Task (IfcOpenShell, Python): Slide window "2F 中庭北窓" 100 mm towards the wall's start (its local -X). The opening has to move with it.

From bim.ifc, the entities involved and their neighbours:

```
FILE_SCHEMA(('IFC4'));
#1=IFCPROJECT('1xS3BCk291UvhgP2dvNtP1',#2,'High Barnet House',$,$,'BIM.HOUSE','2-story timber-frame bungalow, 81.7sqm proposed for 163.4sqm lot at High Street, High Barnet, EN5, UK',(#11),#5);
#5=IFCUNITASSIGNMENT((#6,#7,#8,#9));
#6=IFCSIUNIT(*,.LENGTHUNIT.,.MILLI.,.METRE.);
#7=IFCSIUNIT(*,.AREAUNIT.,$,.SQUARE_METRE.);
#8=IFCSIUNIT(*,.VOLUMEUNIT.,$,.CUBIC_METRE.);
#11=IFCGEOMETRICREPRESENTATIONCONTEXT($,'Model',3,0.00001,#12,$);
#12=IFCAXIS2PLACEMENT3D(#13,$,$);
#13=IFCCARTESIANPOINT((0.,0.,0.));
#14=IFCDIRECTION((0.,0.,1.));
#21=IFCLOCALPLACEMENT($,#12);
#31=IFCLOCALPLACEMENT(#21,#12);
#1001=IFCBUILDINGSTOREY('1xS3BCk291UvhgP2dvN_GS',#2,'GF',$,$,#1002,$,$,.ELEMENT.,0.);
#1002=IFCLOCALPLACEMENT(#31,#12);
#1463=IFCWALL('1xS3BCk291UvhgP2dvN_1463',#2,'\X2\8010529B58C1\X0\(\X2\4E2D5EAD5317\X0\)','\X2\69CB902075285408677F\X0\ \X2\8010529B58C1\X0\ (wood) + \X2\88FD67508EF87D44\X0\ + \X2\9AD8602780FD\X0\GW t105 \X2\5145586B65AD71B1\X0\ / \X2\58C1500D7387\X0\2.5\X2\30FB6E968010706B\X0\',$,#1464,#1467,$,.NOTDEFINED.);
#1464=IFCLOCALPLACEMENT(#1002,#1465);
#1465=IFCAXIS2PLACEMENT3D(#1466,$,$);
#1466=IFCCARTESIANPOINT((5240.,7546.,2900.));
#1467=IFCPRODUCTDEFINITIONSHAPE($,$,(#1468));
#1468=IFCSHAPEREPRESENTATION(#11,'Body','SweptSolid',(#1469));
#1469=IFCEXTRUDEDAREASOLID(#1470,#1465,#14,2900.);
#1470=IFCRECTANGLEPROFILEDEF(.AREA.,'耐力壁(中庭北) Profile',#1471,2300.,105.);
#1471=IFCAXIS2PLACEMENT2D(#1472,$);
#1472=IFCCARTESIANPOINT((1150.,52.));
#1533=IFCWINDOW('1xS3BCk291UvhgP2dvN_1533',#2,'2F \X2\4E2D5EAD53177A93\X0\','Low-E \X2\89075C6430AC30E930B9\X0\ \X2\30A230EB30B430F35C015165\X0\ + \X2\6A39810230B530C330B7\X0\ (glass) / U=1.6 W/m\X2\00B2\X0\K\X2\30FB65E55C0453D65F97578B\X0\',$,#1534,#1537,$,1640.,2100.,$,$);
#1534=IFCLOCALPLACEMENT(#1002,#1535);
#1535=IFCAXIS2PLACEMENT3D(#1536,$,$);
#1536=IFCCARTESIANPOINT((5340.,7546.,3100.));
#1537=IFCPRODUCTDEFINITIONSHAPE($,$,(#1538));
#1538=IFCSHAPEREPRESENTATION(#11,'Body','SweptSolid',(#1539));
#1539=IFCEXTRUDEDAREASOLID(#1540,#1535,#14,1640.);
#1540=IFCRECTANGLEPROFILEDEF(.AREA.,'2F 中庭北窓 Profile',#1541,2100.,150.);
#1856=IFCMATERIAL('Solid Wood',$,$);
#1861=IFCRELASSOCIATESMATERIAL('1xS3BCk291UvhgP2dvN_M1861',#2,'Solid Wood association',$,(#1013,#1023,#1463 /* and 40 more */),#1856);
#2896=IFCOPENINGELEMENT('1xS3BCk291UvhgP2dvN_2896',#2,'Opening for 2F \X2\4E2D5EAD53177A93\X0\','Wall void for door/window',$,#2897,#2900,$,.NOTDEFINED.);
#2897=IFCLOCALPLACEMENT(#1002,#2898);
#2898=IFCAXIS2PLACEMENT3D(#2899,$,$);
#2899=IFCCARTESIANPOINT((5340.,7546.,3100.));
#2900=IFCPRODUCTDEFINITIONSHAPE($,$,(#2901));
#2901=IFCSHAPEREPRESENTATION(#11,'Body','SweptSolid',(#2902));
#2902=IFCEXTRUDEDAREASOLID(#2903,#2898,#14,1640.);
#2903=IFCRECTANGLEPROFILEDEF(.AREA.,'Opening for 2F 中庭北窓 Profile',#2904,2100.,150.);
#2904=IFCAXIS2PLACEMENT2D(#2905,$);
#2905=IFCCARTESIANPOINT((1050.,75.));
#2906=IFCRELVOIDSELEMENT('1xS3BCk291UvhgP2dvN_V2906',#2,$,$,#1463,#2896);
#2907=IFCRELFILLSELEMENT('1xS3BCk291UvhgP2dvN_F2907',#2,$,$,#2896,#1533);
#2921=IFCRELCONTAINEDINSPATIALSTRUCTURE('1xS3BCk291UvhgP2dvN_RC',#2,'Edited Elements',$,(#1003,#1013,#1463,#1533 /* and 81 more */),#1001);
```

```python
import ifcopenshell
import ifcopenshell.api.geometry
import ifcopenshell.util.placement

model = ifcopenshell.open("bim.ifc")

window = model.by_guid("1xS3BCk291UvhgP2dvN_1533")
opening = window.FillsVoids[0].RelatingOpeningElement
wall = opening.VoidsElements[0].RelatingBuildingElement

wall_matrix = ifcopenshell.util.placement.get_local_placement(wall.ObjectPlacement)
shift = wall_matrix[:3, 0] * -100.0
before = ifcopenshell.util.placement.get_local_placement(window.ObjectPlacement)[:3, 3].copy()

# The window is not placed relative to its opening, so move both.
for product in (opening, window):
    matrix = ifcopenshell.util.placement.get_local_placement(product.ObjectPlacement)
    matrix[:3, 3] += shift
    ifcopenshell.api.geometry.edit_object_placement(model, product=product, matrix=matrix, is_si=False)

after = ifcopenshell.util.placement.get_local_placement(window.ObjectPlacement)[:3, 3]
print("window moved by", (after - before).round(3) + 0.0)

model.write("bim_updated.ifc")
```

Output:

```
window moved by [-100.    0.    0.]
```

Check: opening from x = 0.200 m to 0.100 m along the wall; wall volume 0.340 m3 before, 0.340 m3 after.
